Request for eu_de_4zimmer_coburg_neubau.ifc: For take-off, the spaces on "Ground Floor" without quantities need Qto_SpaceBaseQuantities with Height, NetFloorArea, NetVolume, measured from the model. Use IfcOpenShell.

First a look at what the model holds.

```python
import ifcopenshell
import ifcopenshell.util.element
import ifcopenshell.util.unit

model = ifcopenshell.open("eu_de_4zimmer_coburg_neubau.ifc")
print(model.schema)
for unit_type in ("LENGTHUNIT", "AREAUNIT", "VOLUMEUNIT"):
    print(unit_type, ifcopenshell.util.unit.calculate_unit_scale(model, unit_type))
storey = next(s for s in model.by_type("IfcBuildingStorey") if s.Name == "Ground Floor")
spaces = [e for e in ifcopenshell.util.element.get_decomposition(storey) if e.is_a("IfcSpace")]
for e in sorted(spaces, key=lambda e: e.id()):
    print(e.id(), e.is_a(), e.Name, list(ifcopenshell.util.element.get_psets(e, qtos_only=True)), sep=" | ")
```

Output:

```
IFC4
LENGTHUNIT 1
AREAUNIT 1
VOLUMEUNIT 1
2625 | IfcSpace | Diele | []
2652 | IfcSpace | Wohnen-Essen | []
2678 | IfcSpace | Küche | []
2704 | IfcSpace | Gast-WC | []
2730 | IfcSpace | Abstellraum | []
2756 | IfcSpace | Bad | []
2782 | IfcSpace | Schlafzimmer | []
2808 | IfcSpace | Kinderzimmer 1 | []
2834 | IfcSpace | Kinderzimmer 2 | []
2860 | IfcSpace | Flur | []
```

```python
import ifcopenshell
import ifcopenshell.api.pset
import ifcopenshell.geom
import ifcopenshell.util.element
import ifcopenshell.util.shape
import ifcopenshell.util.unit

model = ifcopenshell.open("eu_de_4zimmer_coburg_neubau.ifc")
unit_scale = ifcopenshell.util.unit.calculate_unit_scale(model)
area_scale = ifcopenshell.util.unit.calculate_unit_scale(model, "AREAUNIT")
volume_scale = ifcopenshell.util.unit.calculate_unit_scale(model, "VOLUMEUNIT")
settings = ifcopenshell.geom.settings()

storey = next(s for s in model.by_type("IfcBuildingStorey") if s.Name == "Ground Floor")
spaces = [e for e in ifcopenshell.util.element.get_decomposition(storey) if e.is_a("IfcSpace")]

for e in sorted(spaces, key=lambda e: e.id()):
    if ifcopenshell.util.element.get_psets(e, qtos_only=True, should_inherit=False):
        continue
    # Geometry comes back in metres, in the element's own axes.
    shape = ifcopenshell.geom.create_shape(settings, e)
    values = {
        "Height": ifcopenshell.util.shape.get_z(shape.geometry) / unit_scale,
        "NetFloorArea": ifcopenshell.util.shape.get_footprint_area(shape.geometry) / area_scale,
        "NetVolume": ifcopenshell.util.shape.get_volume(shape.geometry) / volume_scale,
    }
    qto = ifcopenshell.api.pset.add_qto(model, product=e, name="Qto_SpaceBaseQuantities")
    ifcopenshell.api.pset.edit_qto(model, qto=qto, properties=values)
    print(e.id(), {k: round(v, 3) for k, v in values.items()})

model.write("eu_de_4zimmer_coburg_neubau_rev.ifc")
```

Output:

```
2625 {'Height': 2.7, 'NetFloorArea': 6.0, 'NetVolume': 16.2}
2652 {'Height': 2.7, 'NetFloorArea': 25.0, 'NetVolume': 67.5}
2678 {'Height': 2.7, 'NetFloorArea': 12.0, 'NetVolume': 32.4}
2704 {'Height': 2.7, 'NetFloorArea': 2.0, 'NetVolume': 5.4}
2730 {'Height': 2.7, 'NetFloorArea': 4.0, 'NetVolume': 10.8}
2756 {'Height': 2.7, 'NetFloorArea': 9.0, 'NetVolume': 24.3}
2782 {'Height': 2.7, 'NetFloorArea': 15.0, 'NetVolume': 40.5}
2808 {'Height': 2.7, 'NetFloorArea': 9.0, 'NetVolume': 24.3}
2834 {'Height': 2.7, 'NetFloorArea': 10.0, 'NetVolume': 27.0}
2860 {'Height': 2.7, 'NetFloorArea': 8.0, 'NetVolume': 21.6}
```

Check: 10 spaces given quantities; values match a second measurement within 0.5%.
